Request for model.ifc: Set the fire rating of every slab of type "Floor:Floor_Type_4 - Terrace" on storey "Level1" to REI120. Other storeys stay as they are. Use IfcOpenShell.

First a look at what the model holds.

```python
import ifcopenshell
import ifcopenshell.util.element

model = ifcopenshell.open("model.ifc")
print(model.schema)
storey = next(s for s in model.by_type("IfcBuildingStorey") if s.Name == "Level1")
slabs = [e for e in ifcopenshell.util.element.get_decomposition(storey) if e.is_a("IfcSlab")]
seen = {}
for e in slabs:
    element_type = ifcopenshell.util.element.get_type(e)
    key = (element_type.Name if element_type != e and element_type else None, ifcopenshell.util.element.get_pset(e, "Pset_SlabCommon", "FireRating"))
    seen[key] = seen.get(key, 0) + 1
for (name, value), count in sorted(seen.items(), key=str):
    print(count, "x", name, "|", value)
```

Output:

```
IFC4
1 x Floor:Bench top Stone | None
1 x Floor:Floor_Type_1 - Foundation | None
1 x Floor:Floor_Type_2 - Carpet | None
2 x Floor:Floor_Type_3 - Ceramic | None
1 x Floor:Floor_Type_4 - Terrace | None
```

```python
import ifcopenshell
import ifcopenshell.api.pset
import ifcopenshell.util.element

model = ifcopenshell.open("model.ifc")

storey = next(s for s in model.by_type("IfcBuildingStorey") if s.Name == "Level1")
slabs = [e for e in ifcopenshell.util.element.get_decomposition(storey) if e.is_a("IfcSlab")]

count = 0
for e in slabs:
    element_type = ifcopenshell.util.element.get_type(e)
    if element_type in (None, e) or element_type.Name != "Floor:Floor_Type_4 - Terrace":
        continue
    # add_pset returns the element's existing set when there is one.
    pset = ifcopenshell.api.pset.add_pset(model, product=e, name="Pset_SlabCommon")
    ifcopenshell.api.pset.edit_pset(model, pset=pset, properties={"FireRating": "REI120"})
    count += 1

print(count, "slabs updated")

model.write("model-out.ifc")
```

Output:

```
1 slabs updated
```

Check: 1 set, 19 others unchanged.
